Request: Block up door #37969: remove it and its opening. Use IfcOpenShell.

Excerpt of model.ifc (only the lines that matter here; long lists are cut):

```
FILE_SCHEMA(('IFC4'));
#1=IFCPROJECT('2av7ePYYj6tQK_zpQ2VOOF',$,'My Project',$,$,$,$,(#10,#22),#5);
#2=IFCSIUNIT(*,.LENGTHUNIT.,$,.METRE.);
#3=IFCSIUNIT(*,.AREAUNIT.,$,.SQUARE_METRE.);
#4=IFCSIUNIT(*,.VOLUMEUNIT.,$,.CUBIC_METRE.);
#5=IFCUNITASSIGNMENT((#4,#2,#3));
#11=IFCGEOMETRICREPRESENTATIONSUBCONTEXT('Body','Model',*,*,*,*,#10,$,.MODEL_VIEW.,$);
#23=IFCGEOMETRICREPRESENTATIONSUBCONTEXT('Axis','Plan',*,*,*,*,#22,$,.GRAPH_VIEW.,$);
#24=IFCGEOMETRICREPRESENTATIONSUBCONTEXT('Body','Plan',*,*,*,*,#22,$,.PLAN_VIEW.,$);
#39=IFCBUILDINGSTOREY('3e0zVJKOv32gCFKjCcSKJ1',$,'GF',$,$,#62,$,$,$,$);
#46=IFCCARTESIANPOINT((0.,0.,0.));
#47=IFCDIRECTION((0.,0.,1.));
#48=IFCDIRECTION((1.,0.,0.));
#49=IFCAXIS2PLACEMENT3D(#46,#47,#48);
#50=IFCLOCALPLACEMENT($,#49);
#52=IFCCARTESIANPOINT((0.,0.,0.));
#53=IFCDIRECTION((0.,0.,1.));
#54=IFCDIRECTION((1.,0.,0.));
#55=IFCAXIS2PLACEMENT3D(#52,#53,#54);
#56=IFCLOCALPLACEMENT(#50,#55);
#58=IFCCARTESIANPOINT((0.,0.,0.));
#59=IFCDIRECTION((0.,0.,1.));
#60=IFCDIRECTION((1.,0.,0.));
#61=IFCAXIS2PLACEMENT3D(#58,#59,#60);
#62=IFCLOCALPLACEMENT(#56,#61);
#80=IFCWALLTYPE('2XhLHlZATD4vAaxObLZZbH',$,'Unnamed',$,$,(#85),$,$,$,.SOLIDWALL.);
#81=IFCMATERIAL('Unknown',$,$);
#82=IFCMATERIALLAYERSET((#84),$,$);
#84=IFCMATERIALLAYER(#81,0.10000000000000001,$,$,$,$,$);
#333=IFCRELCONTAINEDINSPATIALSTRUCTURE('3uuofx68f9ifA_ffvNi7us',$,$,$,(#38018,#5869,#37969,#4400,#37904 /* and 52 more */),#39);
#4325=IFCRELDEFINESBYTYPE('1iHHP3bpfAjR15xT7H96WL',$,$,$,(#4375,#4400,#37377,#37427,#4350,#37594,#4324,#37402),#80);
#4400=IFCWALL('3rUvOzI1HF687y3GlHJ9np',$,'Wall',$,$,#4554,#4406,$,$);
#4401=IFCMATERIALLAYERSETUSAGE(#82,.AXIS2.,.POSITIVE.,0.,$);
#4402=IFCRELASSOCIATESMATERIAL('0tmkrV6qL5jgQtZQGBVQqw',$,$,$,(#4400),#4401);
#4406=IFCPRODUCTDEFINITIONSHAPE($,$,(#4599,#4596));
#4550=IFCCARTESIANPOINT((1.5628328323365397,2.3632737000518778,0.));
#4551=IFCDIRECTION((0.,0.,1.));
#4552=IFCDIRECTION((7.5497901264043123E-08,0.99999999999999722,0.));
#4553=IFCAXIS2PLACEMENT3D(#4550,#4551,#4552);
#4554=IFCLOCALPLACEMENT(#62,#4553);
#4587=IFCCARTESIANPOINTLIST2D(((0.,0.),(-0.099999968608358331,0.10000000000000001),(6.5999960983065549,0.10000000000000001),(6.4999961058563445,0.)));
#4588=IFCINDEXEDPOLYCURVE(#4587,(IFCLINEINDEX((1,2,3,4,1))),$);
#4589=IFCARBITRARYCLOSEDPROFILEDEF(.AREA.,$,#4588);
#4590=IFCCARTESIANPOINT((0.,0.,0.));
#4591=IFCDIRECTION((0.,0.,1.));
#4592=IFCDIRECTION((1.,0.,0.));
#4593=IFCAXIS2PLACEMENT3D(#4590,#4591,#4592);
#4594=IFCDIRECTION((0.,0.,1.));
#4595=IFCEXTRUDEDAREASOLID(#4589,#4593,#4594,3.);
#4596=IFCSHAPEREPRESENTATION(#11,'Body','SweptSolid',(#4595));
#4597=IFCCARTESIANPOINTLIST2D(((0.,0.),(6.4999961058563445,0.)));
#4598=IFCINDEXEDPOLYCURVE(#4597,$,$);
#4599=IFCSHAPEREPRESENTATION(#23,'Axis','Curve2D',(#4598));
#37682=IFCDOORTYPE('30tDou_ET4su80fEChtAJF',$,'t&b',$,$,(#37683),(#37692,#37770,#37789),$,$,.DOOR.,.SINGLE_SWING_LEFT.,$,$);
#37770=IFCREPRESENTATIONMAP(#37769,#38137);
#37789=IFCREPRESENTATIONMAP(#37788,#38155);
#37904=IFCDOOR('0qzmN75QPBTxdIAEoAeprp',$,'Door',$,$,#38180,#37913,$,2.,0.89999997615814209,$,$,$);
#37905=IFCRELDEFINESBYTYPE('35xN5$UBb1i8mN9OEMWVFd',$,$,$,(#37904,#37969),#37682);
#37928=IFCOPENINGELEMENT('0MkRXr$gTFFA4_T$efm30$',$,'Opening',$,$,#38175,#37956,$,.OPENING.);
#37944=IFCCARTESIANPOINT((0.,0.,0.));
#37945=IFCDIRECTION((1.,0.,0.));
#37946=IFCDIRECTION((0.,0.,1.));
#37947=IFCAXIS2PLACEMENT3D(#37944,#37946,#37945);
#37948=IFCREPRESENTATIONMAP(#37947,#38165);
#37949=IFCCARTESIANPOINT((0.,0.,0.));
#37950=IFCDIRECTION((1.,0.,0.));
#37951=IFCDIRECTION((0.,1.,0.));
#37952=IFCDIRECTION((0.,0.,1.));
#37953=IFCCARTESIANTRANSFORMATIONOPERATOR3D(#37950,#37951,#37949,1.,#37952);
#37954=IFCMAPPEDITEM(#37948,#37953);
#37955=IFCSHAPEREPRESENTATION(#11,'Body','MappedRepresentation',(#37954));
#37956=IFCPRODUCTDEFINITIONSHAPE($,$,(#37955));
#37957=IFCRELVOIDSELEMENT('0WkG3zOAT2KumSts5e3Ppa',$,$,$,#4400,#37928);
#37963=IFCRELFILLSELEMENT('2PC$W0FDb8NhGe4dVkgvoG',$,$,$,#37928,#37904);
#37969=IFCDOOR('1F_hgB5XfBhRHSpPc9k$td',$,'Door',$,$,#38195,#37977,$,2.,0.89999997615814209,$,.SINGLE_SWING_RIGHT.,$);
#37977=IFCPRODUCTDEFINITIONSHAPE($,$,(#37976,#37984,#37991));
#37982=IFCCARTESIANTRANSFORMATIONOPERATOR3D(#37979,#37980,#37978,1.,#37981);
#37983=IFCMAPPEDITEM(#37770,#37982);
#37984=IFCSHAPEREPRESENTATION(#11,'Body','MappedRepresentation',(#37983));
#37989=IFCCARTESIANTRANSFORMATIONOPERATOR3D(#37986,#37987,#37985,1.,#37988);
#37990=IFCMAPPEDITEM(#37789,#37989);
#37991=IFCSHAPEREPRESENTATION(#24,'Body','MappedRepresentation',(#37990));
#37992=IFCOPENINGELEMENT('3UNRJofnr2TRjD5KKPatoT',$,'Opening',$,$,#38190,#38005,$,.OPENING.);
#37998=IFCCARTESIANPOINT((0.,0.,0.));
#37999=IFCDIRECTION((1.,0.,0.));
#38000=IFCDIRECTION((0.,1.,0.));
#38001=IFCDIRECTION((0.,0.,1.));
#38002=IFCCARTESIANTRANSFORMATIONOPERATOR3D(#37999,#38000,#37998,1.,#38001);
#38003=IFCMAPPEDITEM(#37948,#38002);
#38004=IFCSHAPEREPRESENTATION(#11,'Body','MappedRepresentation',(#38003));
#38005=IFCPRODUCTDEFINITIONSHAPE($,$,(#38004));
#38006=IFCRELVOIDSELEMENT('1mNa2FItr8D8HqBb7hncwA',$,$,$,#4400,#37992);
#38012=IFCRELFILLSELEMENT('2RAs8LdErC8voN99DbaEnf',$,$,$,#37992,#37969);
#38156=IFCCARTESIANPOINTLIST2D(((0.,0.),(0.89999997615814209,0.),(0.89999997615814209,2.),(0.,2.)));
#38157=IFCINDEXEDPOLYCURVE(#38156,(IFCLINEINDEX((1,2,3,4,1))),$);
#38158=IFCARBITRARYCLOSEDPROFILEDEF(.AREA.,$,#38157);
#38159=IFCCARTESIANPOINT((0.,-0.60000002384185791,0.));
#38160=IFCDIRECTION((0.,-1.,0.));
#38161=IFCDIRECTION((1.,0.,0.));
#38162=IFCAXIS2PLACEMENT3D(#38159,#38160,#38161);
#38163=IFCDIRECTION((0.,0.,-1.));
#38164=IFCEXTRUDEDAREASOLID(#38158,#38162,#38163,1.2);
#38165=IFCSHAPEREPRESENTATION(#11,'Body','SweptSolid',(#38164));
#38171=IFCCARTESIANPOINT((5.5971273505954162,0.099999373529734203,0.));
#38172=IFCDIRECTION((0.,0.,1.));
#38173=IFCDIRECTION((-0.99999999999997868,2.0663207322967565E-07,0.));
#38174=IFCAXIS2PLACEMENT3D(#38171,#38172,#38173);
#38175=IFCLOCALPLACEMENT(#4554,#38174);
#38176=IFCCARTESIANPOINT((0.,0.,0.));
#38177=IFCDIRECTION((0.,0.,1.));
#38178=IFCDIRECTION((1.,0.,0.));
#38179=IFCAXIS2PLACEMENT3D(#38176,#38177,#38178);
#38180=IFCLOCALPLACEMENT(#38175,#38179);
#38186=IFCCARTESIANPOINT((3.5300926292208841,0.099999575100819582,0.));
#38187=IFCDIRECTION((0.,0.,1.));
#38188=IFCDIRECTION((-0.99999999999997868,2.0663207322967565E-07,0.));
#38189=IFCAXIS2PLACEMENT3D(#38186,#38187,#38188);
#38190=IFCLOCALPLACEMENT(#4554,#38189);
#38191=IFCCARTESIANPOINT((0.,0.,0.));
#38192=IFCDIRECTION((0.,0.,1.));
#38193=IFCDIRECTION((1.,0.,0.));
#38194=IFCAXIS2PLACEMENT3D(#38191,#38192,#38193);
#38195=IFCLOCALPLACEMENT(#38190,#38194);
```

```python
import ifcopenshell
import ifcopenshell.api.feature
import ifcopenshell.api.root
import ifcopenshell.geom
import ifcopenshell.util.shape

model = ifcopenshell.open("model.ifc")
settings = ifcopenshell.geom.settings()


def volume(element):
    """Net volume in cubic metres, openings subtracted."""
    shape = ifcopenshell.geom.create_shape(settings, element)
    return ifcopenshell.util.shape.get_volume(shape.geometry)


door = model.by_guid("1F_hgB5XfBhRHSpPc9k$td")
opening = door.FillsVoids[0].RelatingOpeningElement
wall = opening.VoidsElements[0].RelatingBuildingElement
before = volume(wall)

ifcopenshell.api.root.remove_product(model, product=door)
ifcopenshell.api.feature.remove_feature(model, feature=opening)

after = volume(wall)

print(f"wall volume {before:.3f} -> {after:.3f} m3")

model.write("model_edited.ifc")
```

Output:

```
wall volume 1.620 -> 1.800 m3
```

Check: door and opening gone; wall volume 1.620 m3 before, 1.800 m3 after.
